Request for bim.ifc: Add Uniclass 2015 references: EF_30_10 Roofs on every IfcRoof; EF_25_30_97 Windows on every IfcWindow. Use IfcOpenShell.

First a look at what the model holds.

```python
import ifcopenshell

model = ifcopenshell.open("bim.ifc")
print(model.schema)
print("classifications:", [c.Name for c in model.by_type("IfcClassification")])
for ifc_class in ("IfcDoor", "IfcRoof", "IfcStair", "IfcWall", "IfcWindow"):
    print(ifc_class, len(model.by_type(ifc_class)))
```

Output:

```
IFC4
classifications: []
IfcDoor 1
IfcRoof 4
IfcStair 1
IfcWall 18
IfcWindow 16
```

```python
import ifcopenshell
import ifcopenshell.api.classification

model = ifcopenshell.open("bim.ifc")

system = ifcopenshell.api.classification.add_classification(model, classification="Uniclass 2015")

codes = {
    "IfcRoof": ("EF_30_10", "Roofs"),
    "IfcWindow": ("EF_25_30_97", "Windows"),
}
for ifc_class, (code, name) in codes.items():
    products = model.by_type(ifc_class)
    ifcopenshell.api.classification.add_reference(
        model, products=products, classification=system, identification=code, name=name
    )
    print(code, len(products))

model.write("bim_edited.ifc")
```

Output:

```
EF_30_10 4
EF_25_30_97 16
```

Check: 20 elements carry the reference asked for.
